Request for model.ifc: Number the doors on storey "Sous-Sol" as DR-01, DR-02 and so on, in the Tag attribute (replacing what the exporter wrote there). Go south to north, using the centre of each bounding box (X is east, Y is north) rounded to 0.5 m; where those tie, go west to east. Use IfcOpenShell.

First a look at what the model holds.

```python
import ifcopenshell
import ifcopenshell.util.element
import ifcopenshell.util.placement

model = ifcopenshell.open("model.ifc")
print(model.schema)
storey = next(s for s in model.by_type("IfcBuildingStorey") if s.Name == "Sous-Sol")
doors = [e for e in ifcopenshell.util.element.get_decomposition(storey) if e.is_a("IfcDoor")]
for e in sorted(doors, key=lambda e: e.id()):
    origin = ifcopenshell.util.placement.get_local_placement(e.ObjectPlacement)[:3, 3]
    print(e.id(), e.Tag, e.Name, origin.round(2) + 0.0, sep=" | ")
```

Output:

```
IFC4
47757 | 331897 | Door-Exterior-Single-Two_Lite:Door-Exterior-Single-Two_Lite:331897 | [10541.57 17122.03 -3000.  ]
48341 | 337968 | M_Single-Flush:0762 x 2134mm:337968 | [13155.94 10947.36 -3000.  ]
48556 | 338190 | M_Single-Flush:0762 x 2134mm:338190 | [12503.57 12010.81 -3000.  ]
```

```python
import ifcopenshell
import ifcopenshell.geom
import ifcopenshell.util.element
import ifcopenshell.util.shape

model = ifcopenshell.open("model.ifc")
settings = ifcopenshell.geom.settings()
settings.set("use-world-coords", True)


def centre(element):
    shape = ifcopenshell.geom.create_shape(settings, element)
    return ifcopenshell.util.shape.get_bbox_centroid(shape.geometry)


storey = next(s for s in model.by_type("IfcBuildingStorey") if s.Name == "Sous-Sol")
doors = [e for e in ifcopenshell.util.element.get_decomposition(storey) if e.is_a("IfcDoor")]

# Insertion points can sit at a corner or the storey origin, so sort by the geometry (in metres).
centres = {e: centre(e) for e in doors}
doors.sort(key=lambda e: (round(centres[e][1] / 0.5), centres[e][0]))

for i, e in enumerate(doors, start=1):
    number = f"DR-{i:02d}"
    e.Tag = number
    print(e.id(), number)

model.write("model-out.ifc")
```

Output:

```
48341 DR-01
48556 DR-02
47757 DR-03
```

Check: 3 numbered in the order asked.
